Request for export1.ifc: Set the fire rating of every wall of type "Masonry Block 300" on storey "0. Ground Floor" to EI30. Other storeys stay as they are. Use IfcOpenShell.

First a look at what the model holds.

```python
import ifcopenshell
import ifcopenshell.util.element

model = ifcopenshell.open("export1.ifc")
print(model.schema)
storey = next(s for s in model.by_type("IfcBuildingStorey") if s.Name == "0. Ground Floor")
walls = [e for e in ifcopenshell.util.element.get_decomposition(storey) if e.is_a("IfcWall")]
seen = {}
for e in walls:
    element_type = ifcopenshell.util.element.get_type(e)
    key = (element_type.Name if element_type != e and element_type else None, ifcopenshell.util.element.get_pset(e, "Pset_WallCommon", "FireRating"))
    seen[key] = seen.get(key, 0) + 1
for (name, value), count in sorted(seen.items(), key=str):
    print(count, "x", name, "|", value)
```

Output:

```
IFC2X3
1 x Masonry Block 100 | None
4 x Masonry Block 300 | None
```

```python
import ifcopenshell
import ifcopenshell.api.pset
import ifcopenshell.util.element

model = ifcopenshell.open("export1.ifc")

storey = next(s for s in model.by_type("IfcBuildingStorey") if s.Name == "0. Ground Floor")
walls = [e for e in ifcopenshell.util.element.get_decomposition(storey) if e.is_a("IfcWall")]

count = 0
for e in walls:
    element_type = ifcopenshell.util.element.get_type(e)
    if element_type in (None, e) or element_type.Name != "Masonry Block 300":
        continue
    # add_pset returns the element's existing set when there is one.
    pset = ifcopenshell.api.pset.add_pset(model, product=e, name="Pset_WallCommon")
    ifcopenshell.api.pset.edit_pset(model, pset=pset, properties={"FireRating": "EI30"})
    count += 1

print(count, "walls updated")

model.write("export1_v2.ifc")
```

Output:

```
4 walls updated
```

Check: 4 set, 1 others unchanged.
